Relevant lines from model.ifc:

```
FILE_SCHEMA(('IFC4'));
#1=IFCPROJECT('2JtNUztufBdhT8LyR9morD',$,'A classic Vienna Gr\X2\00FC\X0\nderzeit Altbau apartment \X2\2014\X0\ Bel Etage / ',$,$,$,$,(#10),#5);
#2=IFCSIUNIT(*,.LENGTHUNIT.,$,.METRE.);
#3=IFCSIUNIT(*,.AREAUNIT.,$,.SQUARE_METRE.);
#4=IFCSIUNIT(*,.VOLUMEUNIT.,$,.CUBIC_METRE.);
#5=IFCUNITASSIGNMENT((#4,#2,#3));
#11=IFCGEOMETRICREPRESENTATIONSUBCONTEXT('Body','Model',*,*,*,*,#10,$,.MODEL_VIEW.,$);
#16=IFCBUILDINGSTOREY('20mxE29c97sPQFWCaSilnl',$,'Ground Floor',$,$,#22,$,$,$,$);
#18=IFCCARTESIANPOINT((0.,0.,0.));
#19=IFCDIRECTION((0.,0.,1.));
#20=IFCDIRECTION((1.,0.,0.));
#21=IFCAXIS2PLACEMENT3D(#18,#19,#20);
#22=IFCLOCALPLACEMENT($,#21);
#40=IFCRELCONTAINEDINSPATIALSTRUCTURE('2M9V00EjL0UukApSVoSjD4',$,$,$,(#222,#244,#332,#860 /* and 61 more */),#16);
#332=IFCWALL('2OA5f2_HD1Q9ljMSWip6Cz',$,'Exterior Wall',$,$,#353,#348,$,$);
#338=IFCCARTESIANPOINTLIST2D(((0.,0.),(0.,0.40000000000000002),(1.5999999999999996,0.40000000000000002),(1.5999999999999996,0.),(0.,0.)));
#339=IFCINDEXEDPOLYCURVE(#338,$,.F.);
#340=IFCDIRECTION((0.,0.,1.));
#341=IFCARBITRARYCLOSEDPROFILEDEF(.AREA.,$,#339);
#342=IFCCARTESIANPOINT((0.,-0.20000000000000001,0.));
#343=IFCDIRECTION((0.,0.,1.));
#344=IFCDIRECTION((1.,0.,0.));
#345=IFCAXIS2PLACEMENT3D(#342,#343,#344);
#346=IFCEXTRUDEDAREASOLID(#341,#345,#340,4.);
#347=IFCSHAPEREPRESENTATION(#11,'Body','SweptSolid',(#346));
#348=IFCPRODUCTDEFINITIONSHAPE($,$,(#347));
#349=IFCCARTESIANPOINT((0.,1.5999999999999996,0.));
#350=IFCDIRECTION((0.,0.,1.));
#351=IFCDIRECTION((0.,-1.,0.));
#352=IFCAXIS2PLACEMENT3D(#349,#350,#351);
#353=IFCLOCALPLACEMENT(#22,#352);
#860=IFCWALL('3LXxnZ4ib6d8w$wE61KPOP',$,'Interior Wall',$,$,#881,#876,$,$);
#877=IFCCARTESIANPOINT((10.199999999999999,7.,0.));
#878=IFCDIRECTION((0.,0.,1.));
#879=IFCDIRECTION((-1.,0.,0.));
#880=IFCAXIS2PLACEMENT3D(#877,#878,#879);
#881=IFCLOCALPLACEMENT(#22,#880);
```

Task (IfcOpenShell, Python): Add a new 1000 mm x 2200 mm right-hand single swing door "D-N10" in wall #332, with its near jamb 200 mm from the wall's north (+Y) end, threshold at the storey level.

```python
import numpy as np
import ifcopenshell
import ifcopenshell.api.feature
import ifcopenshell.api.geometry
import ifcopenshell.api.root
import ifcopenshell.api.spatial
import ifcopenshell.geom
import ifcopenshell.util.element
import ifcopenshell.util.placement
import ifcopenshell.util.representation
import ifcopenshell.util.shape
import ifcopenshell.util.unit

model = ifcopenshell.open("model.ifc")
unit_scale = ifcopenshell.util.unit.calculate_unit_scale(model)
settings = ifcopenshell.geom.settings()


def volume(element):
    """Net volume in cubic metres, openings subtracted."""
    shape = ifcopenshell.geom.create_shape(settings, element)
    return ifcopenshell.util.shape.get_volume(shape.geometry)


wall = model.by_id(332)
storey = ifcopenshell.util.element.get_container(wall, ifc_class="IfcBuildingStorey")
context = ifcopenshell.util.representation.get_context(model, "Model", "Body", "MODEL_VIEW")
before = volume(wall)

width, height, from_end, sill = 1, 2.2, 0.2, 0.0  # metres

# The wall runs along its own X axis, and the end named is its -X end.
wall_shape = ifcopenshell.geom.create_shape(settings, wall)
x, y, z = ifcopenshell.util.shape.get_vertices(wall_shape.geometry).T
start = x.min() + from_end
face, thickness = float(y.min()), float(y.max() - y.min())
wall_matrix = ifcopenshell.util.placement.get_local_placement(wall.ObjectPlacement)
level = ifcopenshell.util.placement.get_local_placement(storey.ObjectPlacement)[2, 3]


def in_wall(x, y):
    """Placement at x, y metres in the wall's axes, at sill height."""
    matrix = wall_matrix.copy()
    matrix[:, 3] = wall_matrix @ np.array([x / unit_scale, y / unit_scale, 0.0, 1.0])
    matrix[2, 3] = level + sill / unit_scale
    return matrix


# Opening: a box that overshoots both wall faces by 50 mm.
opening = ifcopenshell.api.root.create_entity(model, ifc_class="IfcOpeningElement", predefined_type="OPENING")
box = ifcopenshell.api.geometry.add_wall_representation(
    model, context=context, length=width, height=height, thickness=thickness + 0.1
)
ifcopenshell.api.geometry.assign_representation(model, product=opening, representation=box)
ifcopenshell.api.geometry.edit_object_placement(model, product=opening, matrix=in_wall(start, face - 0.05), is_si=False)
ifcopenshell.api.feature.add_feature(model, feature=opening, element=wall)

door = ifcopenshell.api.root.create_entity(model, ifc_class="IfcDoor", name="D-N10", predefined_type="DOOR")
door.OverallWidth, door.OverallHeight = width / unit_scale, height / unit_scale
door.OperationType = "SINGLE_SWING_RIGHT"
body = ifcopenshell.api.geometry.add_door_representation(
    model,
    context=context,
    overall_width=door.OverallWidth,
    overall_height=door.OverallHeight,
    operation_type="SINGLE_SWING_RIGHT",
    lining_properties={"LiningDepth": thickness / unit_scale, "ThresholdDepth": thickness / unit_scale},
)
ifcopenshell.api.geometry.assign_representation(model, product=door, representation=body)
ifcopenshell.api.spatial.assign_container(model, products=[door], relating_structure=storey)
ifcopenshell.api.feature.add_filling(model, opening=opening, element=door)

# The lining spans the wall, so the door starts at the wall face.
ifcopenshell.api.geometry.edit_object_placement(model, product=door, matrix=in_wall(start, face), is_si=False)

after = volume(wall)

print(f"wall volume {before:.3f} -> {after:.3f} m3")

model.write("model_edited.ifc")
```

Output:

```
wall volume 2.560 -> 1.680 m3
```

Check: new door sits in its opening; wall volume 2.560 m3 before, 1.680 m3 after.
